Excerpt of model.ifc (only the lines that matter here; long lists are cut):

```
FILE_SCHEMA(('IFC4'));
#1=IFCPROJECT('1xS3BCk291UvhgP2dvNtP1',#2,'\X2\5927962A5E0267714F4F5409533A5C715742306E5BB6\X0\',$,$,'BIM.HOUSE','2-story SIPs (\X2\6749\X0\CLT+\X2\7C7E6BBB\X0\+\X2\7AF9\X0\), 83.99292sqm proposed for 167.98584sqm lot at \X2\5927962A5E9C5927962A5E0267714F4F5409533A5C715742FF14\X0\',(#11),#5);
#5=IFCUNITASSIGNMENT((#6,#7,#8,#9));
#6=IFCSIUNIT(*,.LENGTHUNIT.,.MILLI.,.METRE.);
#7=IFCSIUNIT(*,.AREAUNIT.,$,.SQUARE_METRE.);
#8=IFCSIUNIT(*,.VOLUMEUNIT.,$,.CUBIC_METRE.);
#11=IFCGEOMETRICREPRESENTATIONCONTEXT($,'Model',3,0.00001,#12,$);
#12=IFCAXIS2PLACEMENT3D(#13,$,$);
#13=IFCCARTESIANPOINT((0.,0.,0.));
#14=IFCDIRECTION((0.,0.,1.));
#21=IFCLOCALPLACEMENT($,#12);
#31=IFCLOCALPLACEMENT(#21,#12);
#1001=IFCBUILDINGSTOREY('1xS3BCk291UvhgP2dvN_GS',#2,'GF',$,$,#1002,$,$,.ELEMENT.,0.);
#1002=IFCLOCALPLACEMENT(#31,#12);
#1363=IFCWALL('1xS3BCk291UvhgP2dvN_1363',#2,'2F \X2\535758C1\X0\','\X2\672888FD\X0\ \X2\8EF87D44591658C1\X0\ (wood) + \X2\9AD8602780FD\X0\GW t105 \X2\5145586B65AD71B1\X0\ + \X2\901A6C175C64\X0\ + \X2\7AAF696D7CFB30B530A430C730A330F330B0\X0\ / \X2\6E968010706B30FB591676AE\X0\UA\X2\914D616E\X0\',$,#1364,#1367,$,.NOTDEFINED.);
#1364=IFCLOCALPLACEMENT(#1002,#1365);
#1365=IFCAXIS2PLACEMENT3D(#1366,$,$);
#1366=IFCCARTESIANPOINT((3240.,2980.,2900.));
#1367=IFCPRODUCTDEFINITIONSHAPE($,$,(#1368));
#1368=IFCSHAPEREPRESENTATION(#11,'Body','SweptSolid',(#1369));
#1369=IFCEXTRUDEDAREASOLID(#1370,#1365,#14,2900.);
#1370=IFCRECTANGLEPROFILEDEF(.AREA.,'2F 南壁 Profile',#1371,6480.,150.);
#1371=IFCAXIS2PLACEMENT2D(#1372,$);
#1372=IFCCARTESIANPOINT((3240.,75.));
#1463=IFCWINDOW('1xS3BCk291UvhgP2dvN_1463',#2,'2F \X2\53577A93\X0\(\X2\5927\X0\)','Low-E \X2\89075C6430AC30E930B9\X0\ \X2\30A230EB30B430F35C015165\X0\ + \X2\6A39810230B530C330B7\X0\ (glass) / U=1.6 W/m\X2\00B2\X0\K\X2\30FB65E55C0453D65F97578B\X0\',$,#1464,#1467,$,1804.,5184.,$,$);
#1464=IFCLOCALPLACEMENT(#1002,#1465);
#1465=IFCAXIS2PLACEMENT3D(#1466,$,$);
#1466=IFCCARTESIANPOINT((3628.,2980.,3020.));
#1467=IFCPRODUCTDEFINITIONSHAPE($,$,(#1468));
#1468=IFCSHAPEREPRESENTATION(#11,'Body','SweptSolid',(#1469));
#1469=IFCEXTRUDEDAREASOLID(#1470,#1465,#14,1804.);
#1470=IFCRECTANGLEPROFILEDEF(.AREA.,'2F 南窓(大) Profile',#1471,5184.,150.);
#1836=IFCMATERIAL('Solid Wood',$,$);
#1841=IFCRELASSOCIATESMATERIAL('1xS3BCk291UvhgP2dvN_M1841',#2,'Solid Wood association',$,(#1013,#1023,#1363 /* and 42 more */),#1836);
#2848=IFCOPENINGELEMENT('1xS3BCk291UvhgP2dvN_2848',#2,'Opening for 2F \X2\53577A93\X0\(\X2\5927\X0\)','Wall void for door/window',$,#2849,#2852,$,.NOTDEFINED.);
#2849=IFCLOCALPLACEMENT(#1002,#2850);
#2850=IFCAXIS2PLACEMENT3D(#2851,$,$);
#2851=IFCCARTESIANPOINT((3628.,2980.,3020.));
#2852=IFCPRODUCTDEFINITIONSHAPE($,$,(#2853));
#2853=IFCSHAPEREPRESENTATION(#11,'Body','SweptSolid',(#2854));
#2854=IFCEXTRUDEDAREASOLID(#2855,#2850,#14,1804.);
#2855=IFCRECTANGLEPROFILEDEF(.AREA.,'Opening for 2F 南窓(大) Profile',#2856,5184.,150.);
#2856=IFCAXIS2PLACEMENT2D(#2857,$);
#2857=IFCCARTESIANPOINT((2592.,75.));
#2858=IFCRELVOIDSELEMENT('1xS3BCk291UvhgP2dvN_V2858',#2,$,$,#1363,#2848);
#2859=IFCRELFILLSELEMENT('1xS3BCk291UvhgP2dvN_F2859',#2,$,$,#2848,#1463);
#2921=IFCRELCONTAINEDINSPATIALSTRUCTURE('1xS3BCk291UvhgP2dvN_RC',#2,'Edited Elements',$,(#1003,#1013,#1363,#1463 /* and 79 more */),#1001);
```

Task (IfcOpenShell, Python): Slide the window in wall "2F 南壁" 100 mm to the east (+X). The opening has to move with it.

```python
import ifcopenshell
import ifcopenshell.api.geometry
import ifcopenshell.util.placement
import ifcopenshell.util.unit

model = ifcopenshell.open("model.ifc")
unit_scale = ifcopenshell.util.unit.calculate_unit_scale(model)

window = model.by_guid("1xS3BCk291UvhgP2dvN_1463")
opening = window.FillsVoids[0].RelatingOpeningElement
wall = opening.VoidsElements[0].RelatingBuildingElement

wall_matrix = ifcopenshell.util.placement.get_local_placement(wall.ObjectPlacement)
shift = wall_matrix[:3, 0] * 0.1 / unit_scale
before = ifcopenshell.util.placement.get_local_placement(window.ObjectPlacement)[:3, 3].copy()

# The window is not placed relative to its opening, so move both.
for product in (opening, window):
    matrix = ifcopenshell.util.placement.get_local_placement(product.ObjectPlacement)
    matrix[:3, 3] += shift
    ifcopenshell.api.geometry.edit_object_placement(model, product=product, matrix=matrix, is_si=False)

after = ifcopenshell.util.placement.get_local_placement(window.ObjectPlacement)[:3, 3]
print("window moved by", (after - before).round(3) + 0.0)

model.write("model_rev.ifc")
```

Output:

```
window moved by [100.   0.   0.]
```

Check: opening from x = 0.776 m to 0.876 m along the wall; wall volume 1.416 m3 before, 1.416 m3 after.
